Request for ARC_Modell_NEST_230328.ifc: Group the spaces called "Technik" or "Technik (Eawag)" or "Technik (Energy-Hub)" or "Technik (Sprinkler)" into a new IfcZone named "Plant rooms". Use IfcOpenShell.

First a look at what the model holds.

```python
import ifcopenshell

model = ifcopenshell.open("ARC_Modell_NEST_230328.ifc")
print(model.schema)
seen = {}
for space in model.by_type("IfcSpace"):
    seen[space.LongName] = seen.get(space.LongName, 0) + 1
for name, count in sorted(seen.items(), key=str):
    print(count, "x", name)
print("zones:", [z.Name for z in model.by_type("IfcZone")][:20])
```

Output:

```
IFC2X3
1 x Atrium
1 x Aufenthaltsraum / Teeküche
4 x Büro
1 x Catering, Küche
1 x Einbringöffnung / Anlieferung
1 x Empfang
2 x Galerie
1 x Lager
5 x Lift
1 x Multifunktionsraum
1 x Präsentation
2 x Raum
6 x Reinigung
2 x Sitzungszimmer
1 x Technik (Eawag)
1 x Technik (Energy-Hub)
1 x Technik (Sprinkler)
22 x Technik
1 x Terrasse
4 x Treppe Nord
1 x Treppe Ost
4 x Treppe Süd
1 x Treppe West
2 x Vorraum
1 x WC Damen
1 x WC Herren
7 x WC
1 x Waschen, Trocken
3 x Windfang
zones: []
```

```python
import ifcopenshell
import ifcopenshell.api.group
import ifcopenshell.api.root

model = ifcopenshell.open("ARC_Modell_NEST_230328.ifc")

names = {"Technik", "Technik (Eawag)", "Technik (Energy-Hub)", "Technik (Sprinkler)"}
spaces = [s for s in model.by_type("IfcSpace") if s.LongName in names]

zone = ifcopenshell.api.root.create_entity(model, ifc_class="IfcZone", name="Plant rooms")
ifcopenshell.api.group.assign_group(model, products=spaces, group=zone)
print(len(spaces), "spaces in", zone.Name)

model.write("ARC_Modell_NEST_230328_edited.ifc")
```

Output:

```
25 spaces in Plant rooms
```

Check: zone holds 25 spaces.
